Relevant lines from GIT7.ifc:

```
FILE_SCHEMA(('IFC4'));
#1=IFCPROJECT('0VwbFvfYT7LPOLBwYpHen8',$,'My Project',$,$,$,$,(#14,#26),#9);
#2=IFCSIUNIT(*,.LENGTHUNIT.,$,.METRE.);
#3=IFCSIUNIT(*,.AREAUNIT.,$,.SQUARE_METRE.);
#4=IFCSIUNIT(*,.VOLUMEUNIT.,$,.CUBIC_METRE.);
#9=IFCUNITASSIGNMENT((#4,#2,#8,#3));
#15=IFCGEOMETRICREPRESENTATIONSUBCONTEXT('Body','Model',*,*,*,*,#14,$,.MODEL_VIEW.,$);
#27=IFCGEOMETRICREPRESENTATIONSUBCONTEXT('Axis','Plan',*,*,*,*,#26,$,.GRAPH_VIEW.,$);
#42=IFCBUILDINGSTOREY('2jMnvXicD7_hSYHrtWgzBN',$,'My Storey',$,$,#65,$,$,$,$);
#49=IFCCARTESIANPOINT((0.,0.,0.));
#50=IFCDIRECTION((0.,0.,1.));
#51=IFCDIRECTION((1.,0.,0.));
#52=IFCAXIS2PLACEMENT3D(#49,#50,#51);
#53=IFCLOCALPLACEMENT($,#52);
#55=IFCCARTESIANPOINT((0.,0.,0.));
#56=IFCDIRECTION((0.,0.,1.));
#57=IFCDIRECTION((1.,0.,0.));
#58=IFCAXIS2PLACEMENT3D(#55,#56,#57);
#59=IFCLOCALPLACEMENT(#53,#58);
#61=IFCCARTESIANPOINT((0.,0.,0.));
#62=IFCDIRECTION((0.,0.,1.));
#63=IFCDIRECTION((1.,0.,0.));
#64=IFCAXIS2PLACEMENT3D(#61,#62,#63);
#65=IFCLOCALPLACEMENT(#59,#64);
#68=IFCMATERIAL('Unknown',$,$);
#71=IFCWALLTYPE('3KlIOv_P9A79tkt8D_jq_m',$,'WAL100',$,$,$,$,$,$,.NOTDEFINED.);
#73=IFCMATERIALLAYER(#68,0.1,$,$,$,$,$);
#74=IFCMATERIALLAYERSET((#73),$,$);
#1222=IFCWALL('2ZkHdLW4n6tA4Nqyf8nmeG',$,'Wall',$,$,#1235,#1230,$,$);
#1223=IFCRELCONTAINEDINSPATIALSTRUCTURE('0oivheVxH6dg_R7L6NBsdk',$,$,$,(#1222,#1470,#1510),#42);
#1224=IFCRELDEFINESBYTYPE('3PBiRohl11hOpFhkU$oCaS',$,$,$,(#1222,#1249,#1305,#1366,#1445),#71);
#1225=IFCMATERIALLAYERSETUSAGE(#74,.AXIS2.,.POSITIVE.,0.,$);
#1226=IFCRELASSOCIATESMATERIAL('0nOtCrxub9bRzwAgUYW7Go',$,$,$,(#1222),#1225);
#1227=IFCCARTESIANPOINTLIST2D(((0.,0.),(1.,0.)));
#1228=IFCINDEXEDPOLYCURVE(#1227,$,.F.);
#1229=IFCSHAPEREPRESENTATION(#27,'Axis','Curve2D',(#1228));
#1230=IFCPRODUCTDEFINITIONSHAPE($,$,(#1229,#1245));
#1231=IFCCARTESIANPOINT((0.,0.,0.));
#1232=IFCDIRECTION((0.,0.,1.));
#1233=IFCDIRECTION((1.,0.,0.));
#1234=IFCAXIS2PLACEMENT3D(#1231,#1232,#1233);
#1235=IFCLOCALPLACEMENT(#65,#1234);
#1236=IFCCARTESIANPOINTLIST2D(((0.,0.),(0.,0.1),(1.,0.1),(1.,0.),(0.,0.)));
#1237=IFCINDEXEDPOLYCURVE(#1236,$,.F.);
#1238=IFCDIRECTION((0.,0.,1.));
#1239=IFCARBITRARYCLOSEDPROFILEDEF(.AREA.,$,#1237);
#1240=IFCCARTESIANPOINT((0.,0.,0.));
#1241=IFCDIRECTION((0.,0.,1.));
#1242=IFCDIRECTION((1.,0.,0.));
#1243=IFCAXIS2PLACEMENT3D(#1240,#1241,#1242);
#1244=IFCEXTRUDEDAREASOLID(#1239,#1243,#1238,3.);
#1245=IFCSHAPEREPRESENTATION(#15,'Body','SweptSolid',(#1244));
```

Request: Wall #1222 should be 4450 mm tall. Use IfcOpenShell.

```python
import ifcopenshell
import ifcopenshell.geom
import ifcopenshell.util.representation
import ifcopenshell.util.shape
import ifcopenshell.util.unit

model = ifcopenshell.open("GIT7.ifc")
unit_scale = ifcopenshell.util.unit.calculate_unit_scale(model)
settings = ifcopenshell.geom.settings()


def volume(element):
    """Net volume in cubic metres, openings subtracted."""
    shape = ifcopenshell.geom.create_shape(settings, element)
    return ifcopenshell.util.shape.get_volume(shape.geometry)


wall = model.by_id(1222)
before = volume(wall)

body = ifcopenshell.util.representation.get_representation(wall, "Model", "Body")
solid = body.Items[0]
old_height = solid.Depth
solid.Depth = 4.45 / unit_scale
after = volume(wall)

print(f"height {old_height:g} -> {solid.Depth:g}, volume {before:.3f} -> {after:.3f} m3")

model.write("GIT7_edited.ifc")
```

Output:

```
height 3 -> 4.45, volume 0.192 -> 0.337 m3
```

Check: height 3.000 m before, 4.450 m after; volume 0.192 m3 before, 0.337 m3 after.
